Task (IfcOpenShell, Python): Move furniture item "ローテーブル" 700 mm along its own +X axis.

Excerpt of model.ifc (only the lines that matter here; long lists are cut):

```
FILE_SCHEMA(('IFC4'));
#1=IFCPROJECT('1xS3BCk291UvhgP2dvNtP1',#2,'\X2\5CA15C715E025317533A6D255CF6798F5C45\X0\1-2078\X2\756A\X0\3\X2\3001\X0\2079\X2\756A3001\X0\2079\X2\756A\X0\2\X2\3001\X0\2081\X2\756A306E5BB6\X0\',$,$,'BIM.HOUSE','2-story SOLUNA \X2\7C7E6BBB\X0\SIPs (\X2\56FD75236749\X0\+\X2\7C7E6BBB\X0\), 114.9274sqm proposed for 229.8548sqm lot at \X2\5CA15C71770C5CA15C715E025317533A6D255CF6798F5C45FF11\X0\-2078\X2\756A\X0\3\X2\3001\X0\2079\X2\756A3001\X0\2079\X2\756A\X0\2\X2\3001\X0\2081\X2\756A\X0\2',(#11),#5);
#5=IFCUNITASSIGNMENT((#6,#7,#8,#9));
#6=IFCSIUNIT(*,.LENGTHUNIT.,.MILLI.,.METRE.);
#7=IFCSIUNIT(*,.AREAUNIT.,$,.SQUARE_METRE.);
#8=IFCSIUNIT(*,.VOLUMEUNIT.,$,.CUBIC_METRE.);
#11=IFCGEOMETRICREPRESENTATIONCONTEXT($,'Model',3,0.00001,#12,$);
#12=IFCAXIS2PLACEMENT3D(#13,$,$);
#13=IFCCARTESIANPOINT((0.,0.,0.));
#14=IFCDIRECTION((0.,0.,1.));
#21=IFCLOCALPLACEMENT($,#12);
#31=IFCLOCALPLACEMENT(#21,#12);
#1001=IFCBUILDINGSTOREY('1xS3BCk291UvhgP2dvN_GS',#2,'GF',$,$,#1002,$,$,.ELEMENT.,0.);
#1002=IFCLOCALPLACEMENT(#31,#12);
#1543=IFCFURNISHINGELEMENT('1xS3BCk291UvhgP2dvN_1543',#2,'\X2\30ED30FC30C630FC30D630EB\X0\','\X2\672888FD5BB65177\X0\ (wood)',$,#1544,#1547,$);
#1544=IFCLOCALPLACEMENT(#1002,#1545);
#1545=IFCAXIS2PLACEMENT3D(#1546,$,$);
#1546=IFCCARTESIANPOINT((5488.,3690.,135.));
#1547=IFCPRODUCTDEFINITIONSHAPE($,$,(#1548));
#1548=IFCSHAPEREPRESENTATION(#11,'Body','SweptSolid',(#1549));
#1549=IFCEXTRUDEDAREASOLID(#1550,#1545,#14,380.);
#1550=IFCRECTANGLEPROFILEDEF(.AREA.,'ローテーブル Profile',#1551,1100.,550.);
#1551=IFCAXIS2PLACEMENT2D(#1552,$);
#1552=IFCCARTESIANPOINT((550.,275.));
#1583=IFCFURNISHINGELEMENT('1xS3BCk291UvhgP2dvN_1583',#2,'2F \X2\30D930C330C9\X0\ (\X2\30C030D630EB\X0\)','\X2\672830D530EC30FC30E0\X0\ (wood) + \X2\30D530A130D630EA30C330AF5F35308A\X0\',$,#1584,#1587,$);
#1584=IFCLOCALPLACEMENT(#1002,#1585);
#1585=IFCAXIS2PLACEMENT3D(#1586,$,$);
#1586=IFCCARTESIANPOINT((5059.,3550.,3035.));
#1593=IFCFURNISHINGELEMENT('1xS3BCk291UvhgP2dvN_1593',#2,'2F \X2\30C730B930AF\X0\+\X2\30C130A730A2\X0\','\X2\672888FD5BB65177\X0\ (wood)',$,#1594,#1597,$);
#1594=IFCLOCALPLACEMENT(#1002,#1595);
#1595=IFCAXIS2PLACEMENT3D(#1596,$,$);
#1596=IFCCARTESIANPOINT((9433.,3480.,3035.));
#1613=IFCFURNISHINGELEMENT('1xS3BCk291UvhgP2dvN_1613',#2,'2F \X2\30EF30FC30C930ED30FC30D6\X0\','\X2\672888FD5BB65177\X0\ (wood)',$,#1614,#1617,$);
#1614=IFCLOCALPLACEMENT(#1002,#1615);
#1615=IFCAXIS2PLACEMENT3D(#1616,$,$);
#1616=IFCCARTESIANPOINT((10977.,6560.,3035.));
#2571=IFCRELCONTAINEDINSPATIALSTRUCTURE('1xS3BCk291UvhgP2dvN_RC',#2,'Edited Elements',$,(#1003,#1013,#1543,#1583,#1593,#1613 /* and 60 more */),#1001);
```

```python
import ifcopenshell
import ifcopenshell.api.geometry
import ifcopenshell.util.placement

model = ifcopenshell.open("model.ifc")

item = model.by_guid("1xS3BCk291UvhgP2dvN_1543")
matrix = ifcopenshell.util.placement.get_local_placement(item.ObjectPlacement)
matrix[:3, 3] += matrix[:3, 0] * 700.0
ifcopenshell.api.geometry.edit_object_placement(model, product=item, matrix=matrix, is_si=False)

print(ifcopenshell.util.placement.get_local_placement(item.ObjectPlacement).round(3) + 0.0)

model.write("model_rev.ifc")
```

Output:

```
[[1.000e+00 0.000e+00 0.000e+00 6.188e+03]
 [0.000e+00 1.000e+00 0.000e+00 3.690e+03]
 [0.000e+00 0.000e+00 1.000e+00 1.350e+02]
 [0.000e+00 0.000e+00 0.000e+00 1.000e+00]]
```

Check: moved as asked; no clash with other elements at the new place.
